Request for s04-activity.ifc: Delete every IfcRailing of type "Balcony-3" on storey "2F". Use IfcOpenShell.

First a look at what the model holds.

```python
import ifcopenshell
import ifcopenshell.util.element

model = ifcopenshell.open("s04-activity.ifc")
print(model.schema)
storey = next(s for s in model.by_type("IfcBuildingStorey") if s.Name == "2F")
railings = [e for e in ifcopenshell.util.element.get_decomposition(storey) if e.is_a("IfcRailing")]
seen = {}
for e in railings:
    element_type = ifcopenshell.util.element.get_type(e)
    name = element_type.Name if element_type not in (None, e) else None
    seen[name] = seen.get(name, 0) + 1
for name, count in sorted(seen.items(), key=str):
    print(count, "x", name)
```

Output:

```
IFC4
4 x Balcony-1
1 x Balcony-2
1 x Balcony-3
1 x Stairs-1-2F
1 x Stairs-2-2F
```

```python
import ifcopenshell
import ifcopenshell.api.root
import ifcopenshell.util.element

model = ifcopenshell.open("s04-activity.ifc")

storey = next(s for s in model.by_type("IfcBuildingStorey") if s.Name == "2F")
railings = [e for e in ifcopenshell.util.element.get_decomposition(storey) if e.is_a("IfcRailing")]
targets = [e for e in railings if (t := ifcopenshell.util.element.get_type(e)) not in (None, e) and t.Name == "Balcony-3"]

for e in targets:
    ifcopenshell.api.root.remove_product(model, product=e)
print(len(targets), "removed")

model.write("s04-activity_rev.ifc")
```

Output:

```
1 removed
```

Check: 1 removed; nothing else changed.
